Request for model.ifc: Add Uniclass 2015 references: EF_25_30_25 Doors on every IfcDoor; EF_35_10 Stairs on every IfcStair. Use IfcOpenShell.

First a look at what the model holds.

```python
import ifcopenshell

model = ifcopenshell.open("model.ifc")
print(model.schema)
print("classifications:", [c.Name for c in model.by_type("IfcClassification")])
for ifc_class in ("IfcDoor", "IfcRoof", "IfcStair", "IfcWall", "IfcWindow"):
    print(ifc_class, len(model.by_type(ifc_class)))
```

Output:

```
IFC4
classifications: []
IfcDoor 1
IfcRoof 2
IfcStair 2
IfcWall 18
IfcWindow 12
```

```python
import ifcopenshell
import ifcopenshell.api.classification

model = ifcopenshell.open("model.ifc")

system = ifcopenshell.api.classification.add_classification(model, classification="Uniclass 2015")

codes = {
    "IfcDoor": ("EF_25_30_25", "Doors"),
    "IfcStair": ("EF_35_10", "Stairs"),
}
for ifc_class, (code, name) in codes.items():
    products = model.by_type(ifc_class)
    ifcopenshell.api.classification.add_reference(
        model, products=products, classification=system, identification=code, name=name
    )
    print(code, len(products))

model.write("model_edited.ifc")
```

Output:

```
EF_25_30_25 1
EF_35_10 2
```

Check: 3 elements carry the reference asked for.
